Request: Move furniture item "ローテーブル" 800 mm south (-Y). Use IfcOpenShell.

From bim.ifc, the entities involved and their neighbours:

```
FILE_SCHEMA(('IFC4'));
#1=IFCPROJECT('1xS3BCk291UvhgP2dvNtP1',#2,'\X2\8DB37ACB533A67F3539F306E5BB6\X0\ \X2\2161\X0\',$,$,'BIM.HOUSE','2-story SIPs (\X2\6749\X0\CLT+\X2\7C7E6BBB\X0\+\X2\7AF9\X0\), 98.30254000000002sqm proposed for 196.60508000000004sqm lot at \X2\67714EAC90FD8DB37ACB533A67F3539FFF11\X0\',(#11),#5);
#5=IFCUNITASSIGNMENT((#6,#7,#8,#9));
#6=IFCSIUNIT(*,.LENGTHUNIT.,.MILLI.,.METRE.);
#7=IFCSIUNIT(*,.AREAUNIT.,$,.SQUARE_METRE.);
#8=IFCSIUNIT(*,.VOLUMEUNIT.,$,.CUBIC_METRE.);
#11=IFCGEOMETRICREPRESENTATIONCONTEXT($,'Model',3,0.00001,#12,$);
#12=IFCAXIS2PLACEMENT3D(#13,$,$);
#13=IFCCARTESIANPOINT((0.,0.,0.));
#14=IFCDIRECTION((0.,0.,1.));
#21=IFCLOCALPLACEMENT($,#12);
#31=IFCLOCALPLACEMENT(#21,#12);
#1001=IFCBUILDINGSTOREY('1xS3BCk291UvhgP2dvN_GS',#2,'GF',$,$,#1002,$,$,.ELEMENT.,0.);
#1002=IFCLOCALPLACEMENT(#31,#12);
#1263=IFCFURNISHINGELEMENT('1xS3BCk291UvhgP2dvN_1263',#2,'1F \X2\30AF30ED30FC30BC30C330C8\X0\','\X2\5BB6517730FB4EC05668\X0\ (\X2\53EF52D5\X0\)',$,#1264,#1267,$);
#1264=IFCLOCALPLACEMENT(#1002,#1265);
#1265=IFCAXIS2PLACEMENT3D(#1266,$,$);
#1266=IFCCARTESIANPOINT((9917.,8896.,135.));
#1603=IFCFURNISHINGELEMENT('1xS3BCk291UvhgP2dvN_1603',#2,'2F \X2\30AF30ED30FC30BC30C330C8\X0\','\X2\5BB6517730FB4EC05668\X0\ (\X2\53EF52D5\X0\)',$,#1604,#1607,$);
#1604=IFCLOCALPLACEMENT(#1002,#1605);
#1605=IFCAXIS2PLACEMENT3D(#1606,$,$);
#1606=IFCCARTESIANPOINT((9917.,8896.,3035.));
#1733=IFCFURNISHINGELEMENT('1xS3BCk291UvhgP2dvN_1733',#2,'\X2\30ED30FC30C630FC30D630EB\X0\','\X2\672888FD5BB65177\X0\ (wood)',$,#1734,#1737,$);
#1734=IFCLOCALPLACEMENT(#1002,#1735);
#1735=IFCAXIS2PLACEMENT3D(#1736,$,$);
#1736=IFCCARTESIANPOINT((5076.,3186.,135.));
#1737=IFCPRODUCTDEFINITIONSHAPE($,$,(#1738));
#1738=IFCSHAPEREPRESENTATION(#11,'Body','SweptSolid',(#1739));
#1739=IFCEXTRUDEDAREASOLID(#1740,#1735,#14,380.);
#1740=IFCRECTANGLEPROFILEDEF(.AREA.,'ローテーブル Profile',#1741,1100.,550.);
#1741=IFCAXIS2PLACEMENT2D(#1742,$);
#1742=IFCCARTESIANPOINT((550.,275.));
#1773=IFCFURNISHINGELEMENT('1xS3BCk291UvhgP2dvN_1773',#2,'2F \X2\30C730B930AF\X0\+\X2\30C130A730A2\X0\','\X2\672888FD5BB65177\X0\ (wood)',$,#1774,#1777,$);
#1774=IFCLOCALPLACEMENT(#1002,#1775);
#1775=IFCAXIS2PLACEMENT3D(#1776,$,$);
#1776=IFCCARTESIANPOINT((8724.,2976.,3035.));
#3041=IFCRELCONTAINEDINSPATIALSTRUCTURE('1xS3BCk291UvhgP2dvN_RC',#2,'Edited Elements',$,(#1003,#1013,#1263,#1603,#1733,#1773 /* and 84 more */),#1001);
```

```python
import ifcopenshell
import ifcopenshell.api.geometry
import ifcopenshell.util.placement

model = ifcopenshell.open("bim.ifc")

item = model.by_guid("1xS3BCk291UvhgP2dvN_1733")
matrix = ifcopenshell.util.placement.get_local_placement(item.ObjectPlacement)
matrix[1, 3] -= 800.0
ifcopenshell.api.geometry.edit_object_placement(model, product=item, matrix=matrix, is_si=False)

print(ifcopenshell.util.placement.get_local_placement(item.ObjectPlacement).round(3) + 0.0)

model.write("bim_edited.ifc")
```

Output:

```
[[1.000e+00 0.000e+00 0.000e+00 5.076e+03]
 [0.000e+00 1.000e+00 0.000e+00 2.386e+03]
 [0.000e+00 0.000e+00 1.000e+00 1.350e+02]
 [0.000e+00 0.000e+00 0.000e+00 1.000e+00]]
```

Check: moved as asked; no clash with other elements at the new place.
